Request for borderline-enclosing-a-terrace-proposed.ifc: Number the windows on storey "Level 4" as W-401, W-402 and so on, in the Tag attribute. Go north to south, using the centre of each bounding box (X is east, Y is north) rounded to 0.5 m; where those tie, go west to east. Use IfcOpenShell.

First a look at what the model holds.

```python
import ifcopenshell
import ifcopenshell.util.element
import ifcopenshell.util.placement

model = ifcopenshell.open("borderline-enclosing-a-terrace-proposed.ifc")
print(model.schema)
storey = next(s for s in model.by_type("IfcBuildingStorey") if s.Name == "Level 4")
windows = [e for e in ifcopenshell.util.element.get_decomposition(storey) if e.is_a("IfcWindow")]
for e in sorted(windows, key=lambda e: e.id()):
    origin = ifcopenshell.util.placement.get_local_placement(e.ObjectPlacement)[:3, 3]
    print(e.id(), e.Tag, e.Name, origin.round(2) + 0.0, sep=" | ")
```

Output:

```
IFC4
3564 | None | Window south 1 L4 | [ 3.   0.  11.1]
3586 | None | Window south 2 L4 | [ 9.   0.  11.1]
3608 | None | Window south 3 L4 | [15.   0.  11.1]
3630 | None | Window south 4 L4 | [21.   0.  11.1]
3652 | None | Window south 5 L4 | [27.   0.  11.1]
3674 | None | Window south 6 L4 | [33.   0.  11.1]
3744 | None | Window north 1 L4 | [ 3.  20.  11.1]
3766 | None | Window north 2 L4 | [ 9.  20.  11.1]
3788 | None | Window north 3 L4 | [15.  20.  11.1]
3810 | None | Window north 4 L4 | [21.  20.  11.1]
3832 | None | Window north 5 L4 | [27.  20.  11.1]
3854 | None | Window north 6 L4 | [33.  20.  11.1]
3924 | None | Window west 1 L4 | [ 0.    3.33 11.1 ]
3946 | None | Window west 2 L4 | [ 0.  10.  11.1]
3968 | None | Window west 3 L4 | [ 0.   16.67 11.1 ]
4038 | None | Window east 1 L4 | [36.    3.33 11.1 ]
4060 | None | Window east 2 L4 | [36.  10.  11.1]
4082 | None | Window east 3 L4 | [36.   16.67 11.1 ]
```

```python
import ifcopenshell
import ifcopenshell.geom
import ifcopenshell.util.element
import ifcopenshell.util.shape

model = ifcopenshell.open("borderline-enclosing-a-terrace-proposed.ifc")
settings = ifcopenshell.geom.settings()
settings.set("use-world-coords", True)


def centre(element):
    shape = ifcopenshell.geom.create_shape(settings, element)
    return ifcopenshell.util.shape.get_bbox_centroid(shape.geometry)


storey = next(s for s in model.by_type("IfcBuildingStorey") if s.Name == "Level 4")
windows = [e for e in ifcopenshell.util.element.get_decomposition(storey) if e.is_a("IfcWindow")]

# Insertion points can sit at a corner or the storey origin, so sort by the geometry (in metres).
centres = {e: centre(e) for e in windows}
windows.sort(key=lambda e: (-round(centres[e][1] / 0.5), centres[e][0]))

for i, e in enumerate(windows, start=1):
    number = f"W-4{i:02d}"
    e.Tag = number
    print(e.id(), number)

model.write("borderline-enclosing-a-terrace-proposed_edited.ifc")
```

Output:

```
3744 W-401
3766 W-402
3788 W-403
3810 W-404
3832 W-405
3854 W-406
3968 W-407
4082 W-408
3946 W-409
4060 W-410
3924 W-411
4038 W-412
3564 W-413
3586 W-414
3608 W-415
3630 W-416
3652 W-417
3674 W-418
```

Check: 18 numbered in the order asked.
